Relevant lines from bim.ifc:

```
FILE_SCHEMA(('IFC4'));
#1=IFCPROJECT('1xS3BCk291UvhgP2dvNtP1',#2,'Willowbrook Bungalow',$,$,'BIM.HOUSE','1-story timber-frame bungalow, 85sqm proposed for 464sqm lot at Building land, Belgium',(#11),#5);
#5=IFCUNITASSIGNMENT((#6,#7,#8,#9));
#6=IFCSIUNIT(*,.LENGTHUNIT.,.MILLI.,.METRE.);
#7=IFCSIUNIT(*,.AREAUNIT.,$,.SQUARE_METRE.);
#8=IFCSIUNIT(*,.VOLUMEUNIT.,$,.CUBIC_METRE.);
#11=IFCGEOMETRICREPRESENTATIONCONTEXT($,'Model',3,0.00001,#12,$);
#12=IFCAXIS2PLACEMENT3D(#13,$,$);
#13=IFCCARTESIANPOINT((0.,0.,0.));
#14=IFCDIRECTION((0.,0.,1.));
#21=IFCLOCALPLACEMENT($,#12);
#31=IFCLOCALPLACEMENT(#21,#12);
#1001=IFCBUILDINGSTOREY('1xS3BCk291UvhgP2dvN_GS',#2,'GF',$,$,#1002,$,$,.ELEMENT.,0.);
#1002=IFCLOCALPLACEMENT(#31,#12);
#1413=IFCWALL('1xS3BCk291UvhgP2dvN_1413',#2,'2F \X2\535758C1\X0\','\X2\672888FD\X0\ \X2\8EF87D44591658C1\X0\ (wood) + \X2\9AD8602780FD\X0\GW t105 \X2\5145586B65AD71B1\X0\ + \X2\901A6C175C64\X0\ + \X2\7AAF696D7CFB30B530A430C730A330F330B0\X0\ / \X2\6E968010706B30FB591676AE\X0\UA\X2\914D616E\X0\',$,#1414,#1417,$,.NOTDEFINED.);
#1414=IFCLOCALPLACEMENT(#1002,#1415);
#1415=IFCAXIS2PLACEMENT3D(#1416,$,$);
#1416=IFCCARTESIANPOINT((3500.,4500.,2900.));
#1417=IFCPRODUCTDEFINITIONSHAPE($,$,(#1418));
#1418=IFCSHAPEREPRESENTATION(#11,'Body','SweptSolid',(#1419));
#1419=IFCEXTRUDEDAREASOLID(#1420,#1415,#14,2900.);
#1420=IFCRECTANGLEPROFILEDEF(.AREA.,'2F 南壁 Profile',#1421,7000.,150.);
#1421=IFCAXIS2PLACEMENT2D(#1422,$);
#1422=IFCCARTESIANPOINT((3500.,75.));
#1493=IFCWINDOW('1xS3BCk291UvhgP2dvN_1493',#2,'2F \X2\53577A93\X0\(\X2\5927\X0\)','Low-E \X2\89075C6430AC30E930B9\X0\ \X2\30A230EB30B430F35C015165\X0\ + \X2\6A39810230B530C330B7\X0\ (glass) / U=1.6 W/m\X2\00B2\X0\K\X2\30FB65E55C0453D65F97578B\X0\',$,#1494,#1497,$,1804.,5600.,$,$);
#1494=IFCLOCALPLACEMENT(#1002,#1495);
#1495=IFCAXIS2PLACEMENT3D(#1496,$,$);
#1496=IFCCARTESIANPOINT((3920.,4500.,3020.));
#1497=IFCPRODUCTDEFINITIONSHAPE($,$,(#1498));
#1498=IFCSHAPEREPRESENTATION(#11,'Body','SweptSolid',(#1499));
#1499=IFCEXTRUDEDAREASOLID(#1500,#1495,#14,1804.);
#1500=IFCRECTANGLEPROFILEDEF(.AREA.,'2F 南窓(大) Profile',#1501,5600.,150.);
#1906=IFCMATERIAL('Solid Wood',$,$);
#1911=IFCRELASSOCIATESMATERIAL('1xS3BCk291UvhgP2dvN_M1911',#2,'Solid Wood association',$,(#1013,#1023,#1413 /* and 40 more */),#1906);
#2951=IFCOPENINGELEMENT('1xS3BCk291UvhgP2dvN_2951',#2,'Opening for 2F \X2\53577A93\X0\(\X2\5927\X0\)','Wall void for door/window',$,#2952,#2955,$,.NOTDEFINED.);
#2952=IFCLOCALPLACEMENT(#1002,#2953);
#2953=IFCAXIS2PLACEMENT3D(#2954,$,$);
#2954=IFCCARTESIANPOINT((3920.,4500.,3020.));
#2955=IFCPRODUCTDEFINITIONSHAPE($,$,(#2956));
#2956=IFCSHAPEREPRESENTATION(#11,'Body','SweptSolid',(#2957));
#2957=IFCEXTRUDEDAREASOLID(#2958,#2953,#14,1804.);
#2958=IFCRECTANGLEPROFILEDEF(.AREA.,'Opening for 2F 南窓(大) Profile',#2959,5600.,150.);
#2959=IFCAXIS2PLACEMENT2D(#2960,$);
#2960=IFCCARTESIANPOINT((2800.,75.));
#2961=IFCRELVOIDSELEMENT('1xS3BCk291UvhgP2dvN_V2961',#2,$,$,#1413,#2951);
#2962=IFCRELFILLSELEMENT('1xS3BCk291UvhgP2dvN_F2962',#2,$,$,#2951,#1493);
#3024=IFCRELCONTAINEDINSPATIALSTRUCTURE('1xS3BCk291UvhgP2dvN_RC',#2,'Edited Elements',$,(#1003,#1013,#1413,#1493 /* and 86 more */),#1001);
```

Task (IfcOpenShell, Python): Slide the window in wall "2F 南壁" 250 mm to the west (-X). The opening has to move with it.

```python
import ifcopenshell
import ifcopenshell.api.geometry
import ifcopenshell.util.placement
import ifcopenshell.util.unit

model = ifcopenshell.open("bim.ifc")
unit_scale = ifcopenshell.util.unit.calculate_unit_scale(model)

window = model.by_id(1493)
opening = window.FillsVoids[0].RelatingOpeningElement
wall = opening.VoidsElements[0].RelatingBuildingElement

wall_matrix = ifcopenshell.util.placement.get_local_placement(wall.ObjectPlacement)
shift = wall_matrix[:3, 0] * -0.25 / unit_scale
before = ifcopenshell.util.placement.get_local_placement(window.ObjectPlacement)[:3, 3].copy()

# The window is not placed relative to its opening, so move both.
for product in (opening, window):
    matrix = ifcopenshell.util.placement.get_local_placement(product.ObjectPlacement)
    matrix[:3, 3] += shift
    ifcopenshell.api.geometry.edit_object_placement(model, product=product, matrix=matrix, is_si=False)

after = ifcopenshell.util.placement.get_local_placement(window.ObjectPlacement)[:3, 3]
print("window moved by", (after - before).round(3) + 0.0)

model.write("bim_updated.ifc")
```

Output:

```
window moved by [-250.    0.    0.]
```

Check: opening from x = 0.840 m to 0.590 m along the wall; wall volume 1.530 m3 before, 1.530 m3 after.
